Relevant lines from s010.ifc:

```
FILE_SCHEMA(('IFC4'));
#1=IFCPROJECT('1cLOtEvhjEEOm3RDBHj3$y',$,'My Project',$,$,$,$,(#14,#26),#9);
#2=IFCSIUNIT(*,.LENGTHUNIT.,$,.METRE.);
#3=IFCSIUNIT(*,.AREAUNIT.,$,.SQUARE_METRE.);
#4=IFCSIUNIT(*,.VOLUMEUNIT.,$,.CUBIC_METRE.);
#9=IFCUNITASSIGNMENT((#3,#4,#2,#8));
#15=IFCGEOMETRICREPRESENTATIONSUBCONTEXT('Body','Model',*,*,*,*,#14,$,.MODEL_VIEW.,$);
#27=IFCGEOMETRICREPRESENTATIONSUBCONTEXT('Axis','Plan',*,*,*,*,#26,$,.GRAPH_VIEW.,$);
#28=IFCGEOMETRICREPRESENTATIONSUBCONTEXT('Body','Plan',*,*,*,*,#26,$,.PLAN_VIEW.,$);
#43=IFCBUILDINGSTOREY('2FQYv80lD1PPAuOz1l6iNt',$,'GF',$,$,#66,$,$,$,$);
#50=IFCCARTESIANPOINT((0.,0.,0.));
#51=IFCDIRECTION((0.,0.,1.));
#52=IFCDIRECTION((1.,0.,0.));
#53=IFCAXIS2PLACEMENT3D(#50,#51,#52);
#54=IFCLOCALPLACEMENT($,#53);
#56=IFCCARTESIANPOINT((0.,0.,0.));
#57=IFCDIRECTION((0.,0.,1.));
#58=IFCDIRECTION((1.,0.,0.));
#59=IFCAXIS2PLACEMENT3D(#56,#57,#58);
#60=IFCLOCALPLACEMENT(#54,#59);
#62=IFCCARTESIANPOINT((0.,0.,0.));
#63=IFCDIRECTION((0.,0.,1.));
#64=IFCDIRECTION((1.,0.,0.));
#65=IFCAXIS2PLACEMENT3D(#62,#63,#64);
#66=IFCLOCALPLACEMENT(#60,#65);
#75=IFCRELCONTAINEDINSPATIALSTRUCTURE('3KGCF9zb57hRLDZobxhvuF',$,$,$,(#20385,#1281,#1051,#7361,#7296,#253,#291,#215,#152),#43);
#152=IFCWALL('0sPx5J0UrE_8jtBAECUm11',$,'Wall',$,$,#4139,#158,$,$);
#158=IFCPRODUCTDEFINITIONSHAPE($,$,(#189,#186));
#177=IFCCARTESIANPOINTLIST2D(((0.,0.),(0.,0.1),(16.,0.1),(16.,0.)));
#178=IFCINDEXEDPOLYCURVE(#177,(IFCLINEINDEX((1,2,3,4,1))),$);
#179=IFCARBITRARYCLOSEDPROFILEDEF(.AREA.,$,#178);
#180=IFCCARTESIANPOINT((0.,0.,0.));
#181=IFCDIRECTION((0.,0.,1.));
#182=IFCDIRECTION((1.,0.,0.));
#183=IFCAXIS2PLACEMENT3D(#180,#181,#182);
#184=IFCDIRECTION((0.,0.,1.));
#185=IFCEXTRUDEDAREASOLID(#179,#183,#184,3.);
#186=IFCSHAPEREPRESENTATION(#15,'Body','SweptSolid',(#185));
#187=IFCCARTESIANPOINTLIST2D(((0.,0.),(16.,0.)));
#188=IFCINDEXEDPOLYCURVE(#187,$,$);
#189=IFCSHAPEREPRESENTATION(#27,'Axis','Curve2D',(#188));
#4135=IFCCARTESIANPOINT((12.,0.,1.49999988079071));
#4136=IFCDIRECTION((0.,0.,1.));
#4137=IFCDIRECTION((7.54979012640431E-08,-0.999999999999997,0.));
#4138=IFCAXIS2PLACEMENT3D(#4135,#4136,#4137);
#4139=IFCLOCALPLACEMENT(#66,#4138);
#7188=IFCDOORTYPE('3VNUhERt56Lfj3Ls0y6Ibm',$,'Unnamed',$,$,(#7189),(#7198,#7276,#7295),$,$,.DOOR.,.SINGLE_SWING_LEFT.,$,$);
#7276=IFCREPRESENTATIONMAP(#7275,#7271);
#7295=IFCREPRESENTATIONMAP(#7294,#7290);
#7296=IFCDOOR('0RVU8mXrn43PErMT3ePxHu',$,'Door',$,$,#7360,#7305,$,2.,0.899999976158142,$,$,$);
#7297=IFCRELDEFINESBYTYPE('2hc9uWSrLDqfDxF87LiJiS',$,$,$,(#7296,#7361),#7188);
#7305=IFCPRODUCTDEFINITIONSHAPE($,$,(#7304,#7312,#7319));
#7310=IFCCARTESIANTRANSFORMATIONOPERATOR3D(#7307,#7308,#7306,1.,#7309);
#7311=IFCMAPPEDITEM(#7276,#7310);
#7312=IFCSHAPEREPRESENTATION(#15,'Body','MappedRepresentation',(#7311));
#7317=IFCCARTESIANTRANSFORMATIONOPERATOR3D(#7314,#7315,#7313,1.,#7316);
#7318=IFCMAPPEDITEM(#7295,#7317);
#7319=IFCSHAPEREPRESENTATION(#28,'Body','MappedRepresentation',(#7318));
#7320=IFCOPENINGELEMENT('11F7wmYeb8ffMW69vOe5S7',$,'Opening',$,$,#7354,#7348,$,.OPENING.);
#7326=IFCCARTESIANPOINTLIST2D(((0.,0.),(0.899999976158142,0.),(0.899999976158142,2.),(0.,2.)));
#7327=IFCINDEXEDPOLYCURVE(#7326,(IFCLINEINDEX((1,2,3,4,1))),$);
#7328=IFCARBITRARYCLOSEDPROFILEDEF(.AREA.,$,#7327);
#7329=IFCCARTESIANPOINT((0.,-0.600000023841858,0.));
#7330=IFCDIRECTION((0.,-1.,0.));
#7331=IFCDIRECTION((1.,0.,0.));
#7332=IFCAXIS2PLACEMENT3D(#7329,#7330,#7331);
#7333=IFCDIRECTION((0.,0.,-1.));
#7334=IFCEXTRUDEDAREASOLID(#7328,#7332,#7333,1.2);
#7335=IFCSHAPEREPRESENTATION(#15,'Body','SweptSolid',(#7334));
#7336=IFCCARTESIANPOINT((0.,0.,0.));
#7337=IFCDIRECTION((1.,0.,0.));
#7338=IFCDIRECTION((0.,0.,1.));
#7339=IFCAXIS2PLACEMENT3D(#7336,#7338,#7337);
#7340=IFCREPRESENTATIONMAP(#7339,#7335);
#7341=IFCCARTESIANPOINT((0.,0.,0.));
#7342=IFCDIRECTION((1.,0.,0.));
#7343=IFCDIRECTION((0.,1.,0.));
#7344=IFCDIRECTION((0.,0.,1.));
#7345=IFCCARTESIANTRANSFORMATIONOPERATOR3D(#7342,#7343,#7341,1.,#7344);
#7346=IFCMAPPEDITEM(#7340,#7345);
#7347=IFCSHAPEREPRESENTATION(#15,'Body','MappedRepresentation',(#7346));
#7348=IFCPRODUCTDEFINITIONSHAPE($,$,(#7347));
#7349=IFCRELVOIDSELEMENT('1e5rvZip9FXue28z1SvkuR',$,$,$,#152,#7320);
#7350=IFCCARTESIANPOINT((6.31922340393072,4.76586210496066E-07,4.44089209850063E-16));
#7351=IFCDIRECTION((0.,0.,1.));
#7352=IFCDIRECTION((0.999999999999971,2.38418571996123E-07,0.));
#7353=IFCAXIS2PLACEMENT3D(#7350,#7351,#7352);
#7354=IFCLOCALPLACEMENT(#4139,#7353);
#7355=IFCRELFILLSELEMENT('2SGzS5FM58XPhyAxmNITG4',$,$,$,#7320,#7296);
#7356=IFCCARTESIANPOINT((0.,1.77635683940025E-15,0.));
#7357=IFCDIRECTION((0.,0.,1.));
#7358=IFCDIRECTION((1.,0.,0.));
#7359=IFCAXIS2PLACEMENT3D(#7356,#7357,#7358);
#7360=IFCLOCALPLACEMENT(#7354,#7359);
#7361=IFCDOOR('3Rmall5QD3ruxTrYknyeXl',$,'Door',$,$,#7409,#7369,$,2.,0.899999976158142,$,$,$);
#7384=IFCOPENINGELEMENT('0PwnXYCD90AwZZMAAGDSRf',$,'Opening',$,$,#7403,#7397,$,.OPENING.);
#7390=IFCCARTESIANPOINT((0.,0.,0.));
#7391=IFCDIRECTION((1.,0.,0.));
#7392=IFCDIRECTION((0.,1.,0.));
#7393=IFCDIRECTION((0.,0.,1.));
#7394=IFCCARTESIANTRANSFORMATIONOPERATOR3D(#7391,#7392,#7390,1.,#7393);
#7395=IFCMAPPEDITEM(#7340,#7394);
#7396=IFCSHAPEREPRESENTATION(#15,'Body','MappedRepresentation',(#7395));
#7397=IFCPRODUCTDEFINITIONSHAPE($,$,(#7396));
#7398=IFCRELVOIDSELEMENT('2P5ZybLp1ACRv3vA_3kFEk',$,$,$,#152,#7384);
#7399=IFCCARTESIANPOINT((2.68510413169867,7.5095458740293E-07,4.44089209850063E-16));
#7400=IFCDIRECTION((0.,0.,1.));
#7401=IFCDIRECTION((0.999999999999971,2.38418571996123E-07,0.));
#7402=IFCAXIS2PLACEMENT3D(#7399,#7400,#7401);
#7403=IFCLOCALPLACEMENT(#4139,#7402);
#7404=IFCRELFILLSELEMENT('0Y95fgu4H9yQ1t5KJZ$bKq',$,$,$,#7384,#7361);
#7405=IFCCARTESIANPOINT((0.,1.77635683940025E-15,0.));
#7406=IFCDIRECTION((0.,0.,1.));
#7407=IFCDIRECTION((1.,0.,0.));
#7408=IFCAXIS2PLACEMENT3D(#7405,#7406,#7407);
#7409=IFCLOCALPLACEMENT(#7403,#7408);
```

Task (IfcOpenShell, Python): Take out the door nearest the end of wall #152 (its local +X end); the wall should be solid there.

```python
import ifcopenshell
import ifcopenshell.api.feature
import ifcopenshell.api.root
import ifcopenshell.geom
import ifcopenshell.util.shape

model = ifcopenshell.open("s010.ifc")
settings = ifcopenshell.geom.settings()


def volume(element):
    """Net volume in cubic metres, openings subtracted."""
    shape = ifcopenshell.geom.create_shape(settings, element)
    return ifcopenshell.util.shape.get_volume(shape.geometry)


door = model.by_guid("0RVU8mXrn43PErMT3ePxHu")
opening = door.FillsVoids[0].RelatingOpeningElement
wall = opening.VoidsElements[0].RelatingBuildingElement
before = volume(wall)

ifcopenshell.api.root.remove_product(model, product=door)
ifcopenshell.api.feature.remove_feature(model, feature=opening)

after = volume(wall)

print(f"wall volume {before:.3f} -> {after:.3f} m3")

model.write("s010-out.ifc")
```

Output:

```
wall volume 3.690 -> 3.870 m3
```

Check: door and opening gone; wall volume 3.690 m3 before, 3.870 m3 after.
